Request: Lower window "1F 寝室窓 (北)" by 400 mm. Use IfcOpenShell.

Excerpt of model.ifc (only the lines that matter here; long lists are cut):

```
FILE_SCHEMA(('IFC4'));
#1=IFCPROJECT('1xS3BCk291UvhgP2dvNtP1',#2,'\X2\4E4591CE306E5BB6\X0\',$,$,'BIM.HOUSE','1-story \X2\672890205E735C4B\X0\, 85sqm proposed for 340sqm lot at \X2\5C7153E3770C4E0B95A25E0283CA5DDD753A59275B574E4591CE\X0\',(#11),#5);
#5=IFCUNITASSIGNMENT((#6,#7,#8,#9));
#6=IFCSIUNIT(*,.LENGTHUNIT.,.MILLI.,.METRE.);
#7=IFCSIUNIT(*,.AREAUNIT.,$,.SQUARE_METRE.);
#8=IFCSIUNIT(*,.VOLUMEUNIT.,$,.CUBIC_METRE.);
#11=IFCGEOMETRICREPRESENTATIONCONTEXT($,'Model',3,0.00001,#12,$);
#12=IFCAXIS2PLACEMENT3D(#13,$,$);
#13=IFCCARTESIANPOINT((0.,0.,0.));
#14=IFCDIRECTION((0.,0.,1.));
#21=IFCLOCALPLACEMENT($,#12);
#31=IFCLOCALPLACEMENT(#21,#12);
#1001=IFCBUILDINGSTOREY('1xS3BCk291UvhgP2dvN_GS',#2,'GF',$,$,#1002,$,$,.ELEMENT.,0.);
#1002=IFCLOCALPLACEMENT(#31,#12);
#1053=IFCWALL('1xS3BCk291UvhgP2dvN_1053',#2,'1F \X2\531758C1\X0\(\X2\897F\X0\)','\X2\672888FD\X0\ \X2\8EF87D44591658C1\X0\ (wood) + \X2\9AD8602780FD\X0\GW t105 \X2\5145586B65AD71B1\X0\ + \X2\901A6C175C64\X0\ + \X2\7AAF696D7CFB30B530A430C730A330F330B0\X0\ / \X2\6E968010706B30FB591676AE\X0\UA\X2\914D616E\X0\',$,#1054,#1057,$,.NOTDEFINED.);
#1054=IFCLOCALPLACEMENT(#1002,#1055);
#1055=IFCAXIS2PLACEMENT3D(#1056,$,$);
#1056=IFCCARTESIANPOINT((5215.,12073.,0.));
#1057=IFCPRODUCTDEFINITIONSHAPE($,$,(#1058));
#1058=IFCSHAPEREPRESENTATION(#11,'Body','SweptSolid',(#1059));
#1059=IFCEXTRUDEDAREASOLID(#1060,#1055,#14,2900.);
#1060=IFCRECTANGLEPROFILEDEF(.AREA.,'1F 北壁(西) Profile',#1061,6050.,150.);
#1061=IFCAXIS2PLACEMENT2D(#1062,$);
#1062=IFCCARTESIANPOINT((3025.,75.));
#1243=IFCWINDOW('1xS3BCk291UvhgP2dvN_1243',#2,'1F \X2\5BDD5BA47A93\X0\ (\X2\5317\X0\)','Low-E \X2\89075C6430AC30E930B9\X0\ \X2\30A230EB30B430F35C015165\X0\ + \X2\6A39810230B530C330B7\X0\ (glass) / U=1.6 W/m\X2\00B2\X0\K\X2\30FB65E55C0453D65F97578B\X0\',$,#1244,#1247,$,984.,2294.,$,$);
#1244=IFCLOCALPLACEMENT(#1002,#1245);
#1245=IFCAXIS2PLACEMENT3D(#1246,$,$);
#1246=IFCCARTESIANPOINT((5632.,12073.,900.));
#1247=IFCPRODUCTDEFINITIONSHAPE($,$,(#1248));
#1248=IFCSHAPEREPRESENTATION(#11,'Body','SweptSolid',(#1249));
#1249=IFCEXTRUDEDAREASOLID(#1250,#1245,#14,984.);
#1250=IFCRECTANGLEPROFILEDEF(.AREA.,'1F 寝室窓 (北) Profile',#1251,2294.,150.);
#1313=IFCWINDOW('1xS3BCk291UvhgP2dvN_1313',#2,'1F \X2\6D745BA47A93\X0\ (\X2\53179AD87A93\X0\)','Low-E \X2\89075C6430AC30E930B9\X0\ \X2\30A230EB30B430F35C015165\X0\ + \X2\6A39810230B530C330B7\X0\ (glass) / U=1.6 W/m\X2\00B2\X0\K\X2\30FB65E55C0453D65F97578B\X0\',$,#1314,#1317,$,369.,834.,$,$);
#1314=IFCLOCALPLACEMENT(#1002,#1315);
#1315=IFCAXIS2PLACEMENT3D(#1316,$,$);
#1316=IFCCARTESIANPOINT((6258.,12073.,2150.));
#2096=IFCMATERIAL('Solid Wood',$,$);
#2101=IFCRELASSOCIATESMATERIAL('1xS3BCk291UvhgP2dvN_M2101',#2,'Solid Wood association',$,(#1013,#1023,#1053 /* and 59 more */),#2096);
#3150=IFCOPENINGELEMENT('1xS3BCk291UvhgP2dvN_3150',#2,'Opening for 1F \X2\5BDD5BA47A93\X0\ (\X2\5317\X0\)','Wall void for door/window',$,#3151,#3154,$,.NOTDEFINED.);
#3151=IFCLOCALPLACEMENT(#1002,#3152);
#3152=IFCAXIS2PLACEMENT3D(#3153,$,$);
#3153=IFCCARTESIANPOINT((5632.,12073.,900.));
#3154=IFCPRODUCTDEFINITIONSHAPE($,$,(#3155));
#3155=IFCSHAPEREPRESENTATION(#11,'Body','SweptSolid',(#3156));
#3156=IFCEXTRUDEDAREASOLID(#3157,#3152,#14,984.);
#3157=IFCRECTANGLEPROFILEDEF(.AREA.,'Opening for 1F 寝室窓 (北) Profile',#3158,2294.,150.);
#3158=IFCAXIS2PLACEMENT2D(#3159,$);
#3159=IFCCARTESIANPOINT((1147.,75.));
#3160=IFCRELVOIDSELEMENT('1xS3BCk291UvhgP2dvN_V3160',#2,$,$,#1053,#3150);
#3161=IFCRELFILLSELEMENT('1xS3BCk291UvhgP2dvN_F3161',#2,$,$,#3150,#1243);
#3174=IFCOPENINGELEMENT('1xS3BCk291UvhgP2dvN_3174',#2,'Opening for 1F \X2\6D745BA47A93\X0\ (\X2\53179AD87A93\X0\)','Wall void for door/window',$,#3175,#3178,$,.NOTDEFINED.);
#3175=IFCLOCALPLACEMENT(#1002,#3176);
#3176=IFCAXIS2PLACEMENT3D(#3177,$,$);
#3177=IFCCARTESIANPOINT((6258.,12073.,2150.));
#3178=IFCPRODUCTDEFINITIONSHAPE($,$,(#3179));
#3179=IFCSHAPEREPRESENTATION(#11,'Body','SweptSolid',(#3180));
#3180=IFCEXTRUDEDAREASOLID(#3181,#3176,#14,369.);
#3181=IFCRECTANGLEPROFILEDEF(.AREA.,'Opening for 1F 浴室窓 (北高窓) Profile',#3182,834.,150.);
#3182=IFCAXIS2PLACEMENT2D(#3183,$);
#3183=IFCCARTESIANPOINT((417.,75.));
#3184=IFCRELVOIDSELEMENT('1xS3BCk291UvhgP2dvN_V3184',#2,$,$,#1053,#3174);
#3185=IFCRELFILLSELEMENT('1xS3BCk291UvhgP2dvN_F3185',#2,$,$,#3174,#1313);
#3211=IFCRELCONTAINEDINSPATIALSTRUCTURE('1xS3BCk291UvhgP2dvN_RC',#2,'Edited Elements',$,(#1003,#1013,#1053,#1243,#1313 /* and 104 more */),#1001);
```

```python
import numpy as np
import ifcopenshell
import ifcopenshell.api.geometry
import ifcopenshell.util.placement
import ifcopenshell.util.unit

model = ifcopenshell.open("model.ifc")
unit_scale = ifcopenshell.util.unit.calculate_unit_scale(model)

window = model.by_id(1243)
opening = window.FillsVoids[0].RelatingOpeningElement
dz = -0.4 / unit_scale

shift = np.array([0.0, 0.0, dz])
# The window is not placed relative to its opening, so move both.
for product in (opening, window):
    matrix = ifcopenshell.util.placement.get_local_placement(product.ObjectPlacement)
    matrix[:3, 3] += shift
    ifcopenshell.api.geometry.edit_object_placement(model, product=product, matrix=matrix, is_si=False)

print(f"moved by {dz * unit_scale:+.3f} m")

model.write("model-out.ifc")
```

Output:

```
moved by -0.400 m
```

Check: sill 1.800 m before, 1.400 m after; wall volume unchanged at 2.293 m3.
